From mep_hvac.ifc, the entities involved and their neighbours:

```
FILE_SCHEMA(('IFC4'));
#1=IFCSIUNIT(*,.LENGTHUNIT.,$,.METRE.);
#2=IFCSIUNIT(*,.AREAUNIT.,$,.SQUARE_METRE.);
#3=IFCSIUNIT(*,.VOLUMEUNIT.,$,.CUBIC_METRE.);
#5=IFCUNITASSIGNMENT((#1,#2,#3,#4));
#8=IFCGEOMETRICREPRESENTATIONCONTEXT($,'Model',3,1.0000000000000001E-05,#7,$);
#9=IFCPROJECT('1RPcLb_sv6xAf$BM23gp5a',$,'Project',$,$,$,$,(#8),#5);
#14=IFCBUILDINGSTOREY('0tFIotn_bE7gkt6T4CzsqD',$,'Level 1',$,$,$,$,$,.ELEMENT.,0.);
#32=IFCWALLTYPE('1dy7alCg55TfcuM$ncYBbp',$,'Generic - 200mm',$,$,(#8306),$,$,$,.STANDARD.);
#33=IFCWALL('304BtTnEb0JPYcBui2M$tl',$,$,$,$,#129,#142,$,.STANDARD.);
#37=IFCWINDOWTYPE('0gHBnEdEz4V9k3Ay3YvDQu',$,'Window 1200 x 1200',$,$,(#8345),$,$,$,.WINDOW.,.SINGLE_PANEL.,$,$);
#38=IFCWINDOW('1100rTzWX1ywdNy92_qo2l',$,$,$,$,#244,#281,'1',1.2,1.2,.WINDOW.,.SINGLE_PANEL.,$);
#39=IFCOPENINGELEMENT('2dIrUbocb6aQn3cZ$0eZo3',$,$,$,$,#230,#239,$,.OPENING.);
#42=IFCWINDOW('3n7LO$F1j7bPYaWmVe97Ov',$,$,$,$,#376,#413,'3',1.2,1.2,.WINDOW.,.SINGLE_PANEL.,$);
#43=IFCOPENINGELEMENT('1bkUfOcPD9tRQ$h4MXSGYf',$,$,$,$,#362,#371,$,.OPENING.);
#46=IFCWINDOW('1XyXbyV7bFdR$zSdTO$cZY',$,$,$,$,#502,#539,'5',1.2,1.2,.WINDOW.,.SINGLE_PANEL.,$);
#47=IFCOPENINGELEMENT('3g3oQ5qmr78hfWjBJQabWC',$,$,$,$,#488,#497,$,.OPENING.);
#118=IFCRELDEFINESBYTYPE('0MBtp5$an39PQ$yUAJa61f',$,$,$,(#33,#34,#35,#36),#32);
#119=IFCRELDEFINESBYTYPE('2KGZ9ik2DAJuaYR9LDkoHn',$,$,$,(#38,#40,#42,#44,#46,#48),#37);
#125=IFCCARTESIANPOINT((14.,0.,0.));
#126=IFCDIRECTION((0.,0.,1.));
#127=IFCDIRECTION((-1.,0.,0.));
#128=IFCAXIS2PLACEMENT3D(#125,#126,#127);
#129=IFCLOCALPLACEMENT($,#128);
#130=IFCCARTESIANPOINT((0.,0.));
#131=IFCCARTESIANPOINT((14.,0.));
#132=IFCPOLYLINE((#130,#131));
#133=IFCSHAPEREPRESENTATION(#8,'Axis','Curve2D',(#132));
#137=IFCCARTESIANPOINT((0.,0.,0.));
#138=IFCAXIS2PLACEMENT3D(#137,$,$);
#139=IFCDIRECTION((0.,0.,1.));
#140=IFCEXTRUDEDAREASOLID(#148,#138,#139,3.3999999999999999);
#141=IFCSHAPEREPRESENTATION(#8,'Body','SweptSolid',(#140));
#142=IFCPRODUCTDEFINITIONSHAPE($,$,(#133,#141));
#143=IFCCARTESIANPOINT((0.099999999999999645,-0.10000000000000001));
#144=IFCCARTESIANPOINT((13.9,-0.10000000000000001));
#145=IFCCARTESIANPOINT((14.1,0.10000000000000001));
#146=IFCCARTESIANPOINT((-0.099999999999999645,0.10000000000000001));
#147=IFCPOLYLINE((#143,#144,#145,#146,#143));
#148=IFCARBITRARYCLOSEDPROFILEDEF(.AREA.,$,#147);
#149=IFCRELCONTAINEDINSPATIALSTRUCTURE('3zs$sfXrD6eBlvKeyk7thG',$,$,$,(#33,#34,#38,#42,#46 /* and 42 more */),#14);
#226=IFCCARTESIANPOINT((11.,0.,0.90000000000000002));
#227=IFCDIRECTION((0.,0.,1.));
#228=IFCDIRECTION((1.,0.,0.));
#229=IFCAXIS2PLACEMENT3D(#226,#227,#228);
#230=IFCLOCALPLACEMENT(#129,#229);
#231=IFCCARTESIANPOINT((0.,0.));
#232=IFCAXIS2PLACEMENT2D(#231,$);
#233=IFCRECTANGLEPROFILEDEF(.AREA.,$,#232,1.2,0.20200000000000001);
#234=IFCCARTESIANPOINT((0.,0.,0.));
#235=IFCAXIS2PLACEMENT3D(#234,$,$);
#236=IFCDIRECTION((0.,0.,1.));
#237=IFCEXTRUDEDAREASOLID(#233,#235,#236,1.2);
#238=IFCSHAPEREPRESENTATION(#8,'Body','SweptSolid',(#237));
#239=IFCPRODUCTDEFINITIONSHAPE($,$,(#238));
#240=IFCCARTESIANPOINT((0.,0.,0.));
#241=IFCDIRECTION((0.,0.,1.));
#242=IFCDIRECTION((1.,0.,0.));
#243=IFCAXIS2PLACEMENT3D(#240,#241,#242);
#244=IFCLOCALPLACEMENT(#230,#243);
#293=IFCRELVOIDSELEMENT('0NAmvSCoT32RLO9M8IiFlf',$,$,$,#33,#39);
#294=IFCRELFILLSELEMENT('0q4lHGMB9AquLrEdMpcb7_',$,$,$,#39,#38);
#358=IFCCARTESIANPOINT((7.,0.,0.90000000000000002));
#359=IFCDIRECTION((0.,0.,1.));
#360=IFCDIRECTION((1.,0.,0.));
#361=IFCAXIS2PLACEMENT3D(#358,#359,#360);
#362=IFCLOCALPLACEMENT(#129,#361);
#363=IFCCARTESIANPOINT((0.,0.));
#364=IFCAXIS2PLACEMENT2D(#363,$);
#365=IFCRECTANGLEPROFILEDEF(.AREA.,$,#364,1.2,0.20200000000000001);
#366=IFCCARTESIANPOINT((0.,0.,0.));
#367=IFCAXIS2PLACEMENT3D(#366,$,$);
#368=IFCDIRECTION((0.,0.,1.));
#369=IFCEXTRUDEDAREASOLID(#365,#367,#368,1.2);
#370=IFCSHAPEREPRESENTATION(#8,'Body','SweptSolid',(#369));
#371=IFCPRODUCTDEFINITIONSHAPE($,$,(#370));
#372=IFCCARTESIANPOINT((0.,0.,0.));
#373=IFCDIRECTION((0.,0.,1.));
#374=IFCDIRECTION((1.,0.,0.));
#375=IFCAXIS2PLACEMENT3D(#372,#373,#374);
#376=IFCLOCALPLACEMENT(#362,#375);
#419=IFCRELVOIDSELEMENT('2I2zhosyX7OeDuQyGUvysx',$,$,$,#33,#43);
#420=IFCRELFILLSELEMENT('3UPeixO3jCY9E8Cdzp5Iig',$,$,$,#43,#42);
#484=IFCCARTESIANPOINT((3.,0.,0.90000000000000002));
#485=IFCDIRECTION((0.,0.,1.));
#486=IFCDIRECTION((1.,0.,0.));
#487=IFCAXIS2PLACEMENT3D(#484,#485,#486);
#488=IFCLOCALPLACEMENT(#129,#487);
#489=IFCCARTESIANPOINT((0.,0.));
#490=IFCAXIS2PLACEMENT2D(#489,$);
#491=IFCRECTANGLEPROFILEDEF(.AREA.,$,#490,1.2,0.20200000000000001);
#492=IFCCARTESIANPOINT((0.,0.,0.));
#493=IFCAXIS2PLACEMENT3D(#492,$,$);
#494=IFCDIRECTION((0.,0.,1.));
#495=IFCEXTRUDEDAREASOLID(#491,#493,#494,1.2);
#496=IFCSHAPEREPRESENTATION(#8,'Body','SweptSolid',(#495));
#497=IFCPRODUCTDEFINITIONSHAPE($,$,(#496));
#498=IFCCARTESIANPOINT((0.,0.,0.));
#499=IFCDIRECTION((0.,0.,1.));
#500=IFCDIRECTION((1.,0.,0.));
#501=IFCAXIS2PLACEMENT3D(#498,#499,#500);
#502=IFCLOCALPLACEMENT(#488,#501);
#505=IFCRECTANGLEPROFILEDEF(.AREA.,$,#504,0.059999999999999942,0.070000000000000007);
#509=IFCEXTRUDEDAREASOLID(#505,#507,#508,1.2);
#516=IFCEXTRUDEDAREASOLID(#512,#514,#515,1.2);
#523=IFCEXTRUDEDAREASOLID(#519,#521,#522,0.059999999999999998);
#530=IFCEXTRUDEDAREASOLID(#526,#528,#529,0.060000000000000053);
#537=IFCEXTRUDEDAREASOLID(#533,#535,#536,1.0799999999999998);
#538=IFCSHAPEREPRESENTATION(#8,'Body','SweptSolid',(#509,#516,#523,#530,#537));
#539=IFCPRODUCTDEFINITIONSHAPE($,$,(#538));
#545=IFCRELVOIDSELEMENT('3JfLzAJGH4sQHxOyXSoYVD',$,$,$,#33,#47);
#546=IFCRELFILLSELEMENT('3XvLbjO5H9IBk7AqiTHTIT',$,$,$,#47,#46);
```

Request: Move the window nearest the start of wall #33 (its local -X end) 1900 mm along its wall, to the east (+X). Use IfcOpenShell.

```python
import ifcopenshell
import ifcopenshell.api.geometry
import ifcopenshell.util.placement

model = ifcopenshell.open("mep_hvac.ifc")

window = model.by_guid("1XyXbyV7bFdR$zSdTO$cZY")
opening = window.FillsVoids[0].RelatingOpeningElement
wall = opening.VoidsElements[0].RelatingBuildingElement

wall_matrix = ifcopenshell.util.placement.get_local_placement(wall.ObjectPlacement)
shift = wall_matrix[:3, 0] * -1.9
before = ifcopenshell.util.placement.get_local_placement(window.ObjectPlacement)[:3, 3].copy()

# The window is placed relative to its opening, so it follows when the opening moves.
matrix = ifcopenshell.util.placement.get_local_placement(opening.ObjectPlacement)
matrix[:3, 3] += shift
ifcopenshell.api.geometry.edit_object_placement(
    model, product=opening, matrix=matrix, is_si=False, should_transform_children=True
)

after = ifcopenshell.util.placement.get_local_placement(window.ObjectPlacement)[:3, 3]
print("window moved by", (after - before).round(3) + 0.0)

model.write("mep_hvac_edited.ifc")
```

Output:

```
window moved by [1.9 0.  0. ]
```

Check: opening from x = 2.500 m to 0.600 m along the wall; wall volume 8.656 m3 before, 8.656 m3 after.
